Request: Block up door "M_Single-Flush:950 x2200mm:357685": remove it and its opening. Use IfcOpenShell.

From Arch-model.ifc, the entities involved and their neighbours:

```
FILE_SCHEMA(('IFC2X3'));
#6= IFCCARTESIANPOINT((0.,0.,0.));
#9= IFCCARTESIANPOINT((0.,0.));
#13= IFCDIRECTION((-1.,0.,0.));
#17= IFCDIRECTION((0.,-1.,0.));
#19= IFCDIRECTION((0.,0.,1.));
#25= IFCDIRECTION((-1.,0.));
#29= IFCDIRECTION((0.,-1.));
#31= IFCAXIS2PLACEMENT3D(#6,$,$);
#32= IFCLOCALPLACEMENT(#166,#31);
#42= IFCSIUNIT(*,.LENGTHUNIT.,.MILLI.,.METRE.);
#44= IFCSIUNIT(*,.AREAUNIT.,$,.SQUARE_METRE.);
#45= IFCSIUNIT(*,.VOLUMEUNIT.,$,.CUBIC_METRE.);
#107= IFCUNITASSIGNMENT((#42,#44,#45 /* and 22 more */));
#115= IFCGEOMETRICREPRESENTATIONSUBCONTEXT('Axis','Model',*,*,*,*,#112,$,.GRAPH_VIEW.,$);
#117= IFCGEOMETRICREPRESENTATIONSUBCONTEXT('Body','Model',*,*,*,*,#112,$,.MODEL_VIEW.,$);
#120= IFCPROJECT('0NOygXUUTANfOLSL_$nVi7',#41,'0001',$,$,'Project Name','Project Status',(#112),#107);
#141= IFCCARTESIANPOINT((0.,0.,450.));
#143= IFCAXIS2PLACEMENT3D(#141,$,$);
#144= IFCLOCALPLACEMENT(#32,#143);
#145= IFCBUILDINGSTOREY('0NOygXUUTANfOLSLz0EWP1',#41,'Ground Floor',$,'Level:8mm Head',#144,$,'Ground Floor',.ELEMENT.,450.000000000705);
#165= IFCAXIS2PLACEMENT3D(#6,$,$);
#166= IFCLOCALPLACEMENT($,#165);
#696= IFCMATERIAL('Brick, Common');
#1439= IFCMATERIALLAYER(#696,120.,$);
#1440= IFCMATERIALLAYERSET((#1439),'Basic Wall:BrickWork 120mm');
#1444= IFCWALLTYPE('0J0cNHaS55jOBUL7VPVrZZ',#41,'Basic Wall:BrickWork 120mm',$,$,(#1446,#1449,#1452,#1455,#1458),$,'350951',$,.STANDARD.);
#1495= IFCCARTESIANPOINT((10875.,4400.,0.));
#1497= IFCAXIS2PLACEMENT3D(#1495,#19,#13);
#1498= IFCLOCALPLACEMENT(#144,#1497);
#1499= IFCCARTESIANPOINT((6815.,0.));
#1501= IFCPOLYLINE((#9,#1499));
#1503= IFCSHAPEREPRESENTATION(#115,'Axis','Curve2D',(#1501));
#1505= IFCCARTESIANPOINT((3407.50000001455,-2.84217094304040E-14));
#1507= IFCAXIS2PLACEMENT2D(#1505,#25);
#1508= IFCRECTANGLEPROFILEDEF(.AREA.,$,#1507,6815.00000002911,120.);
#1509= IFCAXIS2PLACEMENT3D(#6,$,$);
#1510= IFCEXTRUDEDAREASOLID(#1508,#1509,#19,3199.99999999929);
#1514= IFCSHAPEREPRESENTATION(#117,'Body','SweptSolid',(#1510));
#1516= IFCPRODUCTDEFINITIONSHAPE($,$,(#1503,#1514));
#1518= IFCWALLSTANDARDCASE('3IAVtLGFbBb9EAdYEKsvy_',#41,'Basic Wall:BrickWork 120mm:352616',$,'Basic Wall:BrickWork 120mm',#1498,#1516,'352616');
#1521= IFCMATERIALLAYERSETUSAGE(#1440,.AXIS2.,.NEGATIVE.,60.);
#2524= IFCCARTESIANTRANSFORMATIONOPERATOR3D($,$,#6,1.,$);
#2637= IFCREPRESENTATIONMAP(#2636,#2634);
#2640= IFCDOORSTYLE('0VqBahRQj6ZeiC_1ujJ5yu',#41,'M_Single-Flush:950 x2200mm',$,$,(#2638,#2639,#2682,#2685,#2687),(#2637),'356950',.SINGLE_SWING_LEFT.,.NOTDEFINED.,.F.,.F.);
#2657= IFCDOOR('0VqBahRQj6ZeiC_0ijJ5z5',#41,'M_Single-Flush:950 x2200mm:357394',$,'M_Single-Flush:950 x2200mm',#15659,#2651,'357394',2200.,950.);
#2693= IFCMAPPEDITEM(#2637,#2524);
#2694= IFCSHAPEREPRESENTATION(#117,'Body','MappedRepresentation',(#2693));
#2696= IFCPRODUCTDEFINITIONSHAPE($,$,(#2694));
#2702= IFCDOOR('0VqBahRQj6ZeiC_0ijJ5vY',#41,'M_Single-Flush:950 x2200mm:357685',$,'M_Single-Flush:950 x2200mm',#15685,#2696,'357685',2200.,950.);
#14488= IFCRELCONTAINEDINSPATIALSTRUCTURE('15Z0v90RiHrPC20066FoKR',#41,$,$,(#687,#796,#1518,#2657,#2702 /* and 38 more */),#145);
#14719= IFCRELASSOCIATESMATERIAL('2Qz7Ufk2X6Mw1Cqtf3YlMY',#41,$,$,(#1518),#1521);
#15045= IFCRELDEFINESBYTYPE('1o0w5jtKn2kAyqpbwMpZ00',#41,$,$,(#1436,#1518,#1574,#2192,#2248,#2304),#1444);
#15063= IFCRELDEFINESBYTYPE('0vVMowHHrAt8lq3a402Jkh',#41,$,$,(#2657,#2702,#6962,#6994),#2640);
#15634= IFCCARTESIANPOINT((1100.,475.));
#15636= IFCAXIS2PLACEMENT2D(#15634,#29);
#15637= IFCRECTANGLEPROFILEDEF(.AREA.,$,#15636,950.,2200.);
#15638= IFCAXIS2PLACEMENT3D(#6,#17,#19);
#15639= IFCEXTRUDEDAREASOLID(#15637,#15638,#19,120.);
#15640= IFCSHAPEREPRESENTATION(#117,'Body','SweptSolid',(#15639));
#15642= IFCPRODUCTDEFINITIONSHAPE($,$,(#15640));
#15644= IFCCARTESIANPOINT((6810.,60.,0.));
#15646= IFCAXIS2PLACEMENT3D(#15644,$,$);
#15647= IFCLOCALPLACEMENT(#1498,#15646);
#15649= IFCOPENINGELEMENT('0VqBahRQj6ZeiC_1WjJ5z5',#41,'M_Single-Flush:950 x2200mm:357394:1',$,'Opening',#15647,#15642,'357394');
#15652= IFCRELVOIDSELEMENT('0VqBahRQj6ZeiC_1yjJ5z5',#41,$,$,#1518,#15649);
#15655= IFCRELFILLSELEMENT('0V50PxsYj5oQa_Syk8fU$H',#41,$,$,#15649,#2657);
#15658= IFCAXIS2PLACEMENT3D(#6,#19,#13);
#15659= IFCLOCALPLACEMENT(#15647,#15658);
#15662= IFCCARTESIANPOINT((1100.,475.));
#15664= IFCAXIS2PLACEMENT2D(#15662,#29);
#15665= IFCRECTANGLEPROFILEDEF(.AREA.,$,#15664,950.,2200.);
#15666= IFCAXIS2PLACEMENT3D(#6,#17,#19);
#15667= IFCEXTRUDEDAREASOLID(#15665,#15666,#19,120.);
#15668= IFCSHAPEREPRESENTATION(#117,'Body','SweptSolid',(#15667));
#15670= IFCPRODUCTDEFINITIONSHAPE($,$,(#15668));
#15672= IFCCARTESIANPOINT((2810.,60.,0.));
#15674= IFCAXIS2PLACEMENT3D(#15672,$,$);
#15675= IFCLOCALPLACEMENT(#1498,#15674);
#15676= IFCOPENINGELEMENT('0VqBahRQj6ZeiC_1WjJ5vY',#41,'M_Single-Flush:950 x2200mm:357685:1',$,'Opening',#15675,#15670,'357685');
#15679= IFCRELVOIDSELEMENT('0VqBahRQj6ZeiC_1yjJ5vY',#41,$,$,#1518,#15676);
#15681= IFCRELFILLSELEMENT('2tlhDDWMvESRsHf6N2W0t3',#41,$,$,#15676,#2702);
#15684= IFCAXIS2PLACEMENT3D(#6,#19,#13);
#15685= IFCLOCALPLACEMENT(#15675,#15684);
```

```python
import ifcopenshell
import ifcopenshell.api.feature
import ifcopenshell.api.root
import ifcopenshell.geom
import ifcopenshell.util.shape

model = ifcopenshell.open("Arch-model.ifc")
settings = ifcopenshell.geom.settings()


def volume(element):
    """Net volume in cubic metres, openings subtracted."""
    shape = ifcopenshell.geom.create_shape(settings, element)
    return ifcopenshell.util.shape.get_volume(shape.geometry)


door = model.by_guid("0VqBahRQj6ZeiC_0ijJ5vY")
opening = door.FillsVoids[0].RelatingOpeningElement
wall = opening.VoidsElements[0].RelatingBuildingElement
before = volume(wall)

ifcopenshell.api.root.remove_product(model, product=door)
ifcopenshell.api.feature.remove_feature(model, feature=opening)

after = volume(wall)

print(f"wall volume {before:.3f} -> {after:.3f} m3")

model.write("Arch-model_updated.ifc")
```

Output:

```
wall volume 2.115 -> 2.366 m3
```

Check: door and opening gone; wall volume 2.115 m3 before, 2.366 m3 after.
